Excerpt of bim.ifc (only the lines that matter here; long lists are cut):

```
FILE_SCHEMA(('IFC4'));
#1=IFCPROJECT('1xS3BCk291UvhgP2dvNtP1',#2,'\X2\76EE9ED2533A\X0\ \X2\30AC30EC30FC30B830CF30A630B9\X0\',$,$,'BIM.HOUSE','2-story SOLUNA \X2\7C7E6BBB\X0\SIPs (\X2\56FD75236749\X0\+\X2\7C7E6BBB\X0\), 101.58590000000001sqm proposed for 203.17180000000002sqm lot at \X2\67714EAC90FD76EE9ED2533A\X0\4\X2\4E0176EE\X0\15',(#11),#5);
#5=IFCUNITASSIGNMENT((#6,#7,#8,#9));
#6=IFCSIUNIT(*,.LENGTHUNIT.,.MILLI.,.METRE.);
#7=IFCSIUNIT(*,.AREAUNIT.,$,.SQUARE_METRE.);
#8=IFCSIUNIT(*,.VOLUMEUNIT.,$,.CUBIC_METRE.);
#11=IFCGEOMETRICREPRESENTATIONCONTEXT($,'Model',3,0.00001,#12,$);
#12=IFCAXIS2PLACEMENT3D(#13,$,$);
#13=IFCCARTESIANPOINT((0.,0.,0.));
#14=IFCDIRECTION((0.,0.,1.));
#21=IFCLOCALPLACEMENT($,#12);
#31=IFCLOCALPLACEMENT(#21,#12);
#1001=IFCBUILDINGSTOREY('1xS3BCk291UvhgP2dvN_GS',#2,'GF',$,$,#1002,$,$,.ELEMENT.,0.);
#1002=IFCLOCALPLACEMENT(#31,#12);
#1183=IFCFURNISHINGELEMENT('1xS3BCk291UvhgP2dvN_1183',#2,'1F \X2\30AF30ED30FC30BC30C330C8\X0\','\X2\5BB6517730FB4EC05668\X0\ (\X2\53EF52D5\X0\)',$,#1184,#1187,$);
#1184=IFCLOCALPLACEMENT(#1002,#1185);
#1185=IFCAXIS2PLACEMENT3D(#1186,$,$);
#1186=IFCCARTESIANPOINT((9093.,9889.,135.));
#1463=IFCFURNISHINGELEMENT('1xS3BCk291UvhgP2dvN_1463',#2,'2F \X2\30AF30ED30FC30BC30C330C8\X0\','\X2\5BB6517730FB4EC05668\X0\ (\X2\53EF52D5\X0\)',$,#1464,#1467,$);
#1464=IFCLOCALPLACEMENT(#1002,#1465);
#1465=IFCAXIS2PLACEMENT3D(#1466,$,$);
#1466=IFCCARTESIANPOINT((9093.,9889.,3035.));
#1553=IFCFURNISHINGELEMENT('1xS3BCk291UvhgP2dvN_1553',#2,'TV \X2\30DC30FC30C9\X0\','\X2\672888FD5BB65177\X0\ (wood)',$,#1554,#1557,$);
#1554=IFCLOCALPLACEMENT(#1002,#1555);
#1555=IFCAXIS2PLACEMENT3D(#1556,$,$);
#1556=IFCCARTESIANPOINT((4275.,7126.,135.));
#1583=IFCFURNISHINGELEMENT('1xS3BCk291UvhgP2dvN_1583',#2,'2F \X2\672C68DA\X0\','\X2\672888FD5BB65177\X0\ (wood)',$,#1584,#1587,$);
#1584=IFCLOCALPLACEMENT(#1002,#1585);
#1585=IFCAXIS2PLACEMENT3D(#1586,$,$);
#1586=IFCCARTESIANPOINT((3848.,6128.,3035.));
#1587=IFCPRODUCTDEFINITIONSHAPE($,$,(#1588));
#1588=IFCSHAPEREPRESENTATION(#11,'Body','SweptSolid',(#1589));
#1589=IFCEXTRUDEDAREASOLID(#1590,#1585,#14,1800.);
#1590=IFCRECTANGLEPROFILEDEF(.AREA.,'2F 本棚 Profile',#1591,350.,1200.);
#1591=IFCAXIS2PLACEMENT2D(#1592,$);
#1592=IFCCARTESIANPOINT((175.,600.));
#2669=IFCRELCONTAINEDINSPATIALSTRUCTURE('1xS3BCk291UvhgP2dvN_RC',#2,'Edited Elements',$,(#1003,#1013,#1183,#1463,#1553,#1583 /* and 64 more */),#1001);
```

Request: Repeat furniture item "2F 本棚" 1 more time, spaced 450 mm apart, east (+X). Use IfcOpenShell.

```python
import numpy as np
import ifcopenshell
import ifcopenshell.api.geometry
import ifcopenshell.api.root
import ifcopenshell.util.element
import ifcopenshell.util.placement

model = ifcopenshell.open("bim.ifc")


def reuse_history(source, copy):
    """copy_class also copies each property set's owner history, people and application; keep the originals."""
    for rel in copy.IsDefinedBy:
        if rel.is_a("IfcRelDefinesByProperties") and (history := rel.RelatingPropertyDefinition.OwnerHistory):
            rel.RelatingPropertyDefinition.OwnerHistory = source.OwnerHistory
            ifcopenshell.util.element.remove_deep2(model, history)


source = model.by_guid("1xS3BCk291UvhgP2dvN_1583")
base = ifcopenshell.util.placement.get_local_placement(source.ObjectPlacement)
step = np.array([1.0, 0.0, 0.0]) * 450.0

for i in range(1, 2):
    copy = ifcopenshell.api.root.copy_class(model, product=source)
    copy.Representation = ifcopenshell.util.element.copy_deep(
        model, source.Representation, exclude=["IfcGeometricRepresentationContext", "IfcRepresentationMap"]
    )
    reuse_history(source, copy)
    matrix = base.copy()
    matrix[:3, 3] += i * step
    print("added at", matrix[:3, 3].round(3) + 0.0)
    ifcopenshell.api.geometry.edit_object_placement(model, product=copy, matrix=matrix, is_si=False)

model.write("bim-out.ifc")
```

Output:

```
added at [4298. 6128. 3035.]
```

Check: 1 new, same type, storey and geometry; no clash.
